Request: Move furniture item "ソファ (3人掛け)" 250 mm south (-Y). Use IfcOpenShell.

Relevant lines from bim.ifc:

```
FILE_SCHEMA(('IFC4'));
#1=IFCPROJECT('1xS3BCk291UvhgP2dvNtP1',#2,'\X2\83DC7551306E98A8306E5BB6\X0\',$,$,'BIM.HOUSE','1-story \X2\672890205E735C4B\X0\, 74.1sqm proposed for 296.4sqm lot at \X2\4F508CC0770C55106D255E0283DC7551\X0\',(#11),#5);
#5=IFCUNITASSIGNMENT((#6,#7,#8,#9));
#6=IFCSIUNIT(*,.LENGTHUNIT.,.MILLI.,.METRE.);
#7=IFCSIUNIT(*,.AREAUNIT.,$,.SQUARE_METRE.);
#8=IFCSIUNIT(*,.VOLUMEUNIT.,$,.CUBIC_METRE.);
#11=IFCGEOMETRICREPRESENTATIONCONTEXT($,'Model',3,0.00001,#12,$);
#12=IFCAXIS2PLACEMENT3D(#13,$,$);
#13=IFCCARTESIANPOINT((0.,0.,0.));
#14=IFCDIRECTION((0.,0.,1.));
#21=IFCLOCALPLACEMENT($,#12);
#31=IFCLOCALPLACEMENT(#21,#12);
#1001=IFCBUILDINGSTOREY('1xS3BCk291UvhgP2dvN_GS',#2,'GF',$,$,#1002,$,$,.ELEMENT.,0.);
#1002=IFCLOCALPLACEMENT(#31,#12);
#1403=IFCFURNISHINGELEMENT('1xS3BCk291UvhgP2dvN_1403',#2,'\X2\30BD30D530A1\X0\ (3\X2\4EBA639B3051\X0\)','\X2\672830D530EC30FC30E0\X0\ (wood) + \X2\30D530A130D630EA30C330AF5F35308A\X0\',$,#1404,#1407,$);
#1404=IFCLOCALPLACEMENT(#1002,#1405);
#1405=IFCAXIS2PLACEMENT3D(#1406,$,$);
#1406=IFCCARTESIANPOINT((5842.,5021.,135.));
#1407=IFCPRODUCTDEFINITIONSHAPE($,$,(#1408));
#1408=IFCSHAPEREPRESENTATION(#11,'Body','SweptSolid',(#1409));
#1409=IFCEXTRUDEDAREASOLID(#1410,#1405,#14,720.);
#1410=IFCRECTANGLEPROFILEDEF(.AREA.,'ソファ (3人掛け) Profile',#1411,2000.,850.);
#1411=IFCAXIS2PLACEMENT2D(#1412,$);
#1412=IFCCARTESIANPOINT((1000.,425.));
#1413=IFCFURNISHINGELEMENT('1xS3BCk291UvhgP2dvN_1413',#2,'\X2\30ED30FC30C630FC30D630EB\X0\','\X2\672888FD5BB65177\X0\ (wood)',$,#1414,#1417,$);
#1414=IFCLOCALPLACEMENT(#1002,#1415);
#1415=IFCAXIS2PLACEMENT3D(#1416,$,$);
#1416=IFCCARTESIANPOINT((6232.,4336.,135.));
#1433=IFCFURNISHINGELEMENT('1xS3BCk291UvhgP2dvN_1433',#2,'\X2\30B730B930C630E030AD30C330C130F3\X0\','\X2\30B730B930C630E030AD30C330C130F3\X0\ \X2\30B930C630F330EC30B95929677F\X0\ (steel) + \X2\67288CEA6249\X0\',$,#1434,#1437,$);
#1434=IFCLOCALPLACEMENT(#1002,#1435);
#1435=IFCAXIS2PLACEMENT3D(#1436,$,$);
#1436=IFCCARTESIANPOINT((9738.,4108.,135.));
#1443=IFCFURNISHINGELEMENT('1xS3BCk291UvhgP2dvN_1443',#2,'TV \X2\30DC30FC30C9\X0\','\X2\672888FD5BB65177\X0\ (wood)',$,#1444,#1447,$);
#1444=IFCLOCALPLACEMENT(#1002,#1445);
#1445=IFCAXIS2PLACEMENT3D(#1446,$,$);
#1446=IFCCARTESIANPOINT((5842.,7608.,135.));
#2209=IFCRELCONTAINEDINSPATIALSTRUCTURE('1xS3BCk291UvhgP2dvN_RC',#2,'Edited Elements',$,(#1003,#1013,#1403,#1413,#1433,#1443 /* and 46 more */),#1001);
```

```python
import ifcopenshell
import ifcopenshell.api.geometry
import ifcopenshell.util.placement

model = ifcopenshell.open("bim.ifc")

item = model.by_guid("1xS3BCk291UvhgP2dvN_1403")
matrix = ifcopenshell.util.placement.get_local_placement(item.ObjectPlacement)
matrix[1, 3] -= 250.0
ifcopenshell.api.geometry.edit_object_placement(model, product=item, matrix=matrix, is_si=False)

print(ifcopenshell.util.placement.get_local_placement(item.ObjectPlacement).round(3) + 0.0)

model.write("bim_edited.ifc")
```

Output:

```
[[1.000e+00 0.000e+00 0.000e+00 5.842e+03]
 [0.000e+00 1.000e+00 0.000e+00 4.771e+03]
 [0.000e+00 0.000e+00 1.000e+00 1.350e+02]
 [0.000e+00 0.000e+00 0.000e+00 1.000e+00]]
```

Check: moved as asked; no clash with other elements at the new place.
